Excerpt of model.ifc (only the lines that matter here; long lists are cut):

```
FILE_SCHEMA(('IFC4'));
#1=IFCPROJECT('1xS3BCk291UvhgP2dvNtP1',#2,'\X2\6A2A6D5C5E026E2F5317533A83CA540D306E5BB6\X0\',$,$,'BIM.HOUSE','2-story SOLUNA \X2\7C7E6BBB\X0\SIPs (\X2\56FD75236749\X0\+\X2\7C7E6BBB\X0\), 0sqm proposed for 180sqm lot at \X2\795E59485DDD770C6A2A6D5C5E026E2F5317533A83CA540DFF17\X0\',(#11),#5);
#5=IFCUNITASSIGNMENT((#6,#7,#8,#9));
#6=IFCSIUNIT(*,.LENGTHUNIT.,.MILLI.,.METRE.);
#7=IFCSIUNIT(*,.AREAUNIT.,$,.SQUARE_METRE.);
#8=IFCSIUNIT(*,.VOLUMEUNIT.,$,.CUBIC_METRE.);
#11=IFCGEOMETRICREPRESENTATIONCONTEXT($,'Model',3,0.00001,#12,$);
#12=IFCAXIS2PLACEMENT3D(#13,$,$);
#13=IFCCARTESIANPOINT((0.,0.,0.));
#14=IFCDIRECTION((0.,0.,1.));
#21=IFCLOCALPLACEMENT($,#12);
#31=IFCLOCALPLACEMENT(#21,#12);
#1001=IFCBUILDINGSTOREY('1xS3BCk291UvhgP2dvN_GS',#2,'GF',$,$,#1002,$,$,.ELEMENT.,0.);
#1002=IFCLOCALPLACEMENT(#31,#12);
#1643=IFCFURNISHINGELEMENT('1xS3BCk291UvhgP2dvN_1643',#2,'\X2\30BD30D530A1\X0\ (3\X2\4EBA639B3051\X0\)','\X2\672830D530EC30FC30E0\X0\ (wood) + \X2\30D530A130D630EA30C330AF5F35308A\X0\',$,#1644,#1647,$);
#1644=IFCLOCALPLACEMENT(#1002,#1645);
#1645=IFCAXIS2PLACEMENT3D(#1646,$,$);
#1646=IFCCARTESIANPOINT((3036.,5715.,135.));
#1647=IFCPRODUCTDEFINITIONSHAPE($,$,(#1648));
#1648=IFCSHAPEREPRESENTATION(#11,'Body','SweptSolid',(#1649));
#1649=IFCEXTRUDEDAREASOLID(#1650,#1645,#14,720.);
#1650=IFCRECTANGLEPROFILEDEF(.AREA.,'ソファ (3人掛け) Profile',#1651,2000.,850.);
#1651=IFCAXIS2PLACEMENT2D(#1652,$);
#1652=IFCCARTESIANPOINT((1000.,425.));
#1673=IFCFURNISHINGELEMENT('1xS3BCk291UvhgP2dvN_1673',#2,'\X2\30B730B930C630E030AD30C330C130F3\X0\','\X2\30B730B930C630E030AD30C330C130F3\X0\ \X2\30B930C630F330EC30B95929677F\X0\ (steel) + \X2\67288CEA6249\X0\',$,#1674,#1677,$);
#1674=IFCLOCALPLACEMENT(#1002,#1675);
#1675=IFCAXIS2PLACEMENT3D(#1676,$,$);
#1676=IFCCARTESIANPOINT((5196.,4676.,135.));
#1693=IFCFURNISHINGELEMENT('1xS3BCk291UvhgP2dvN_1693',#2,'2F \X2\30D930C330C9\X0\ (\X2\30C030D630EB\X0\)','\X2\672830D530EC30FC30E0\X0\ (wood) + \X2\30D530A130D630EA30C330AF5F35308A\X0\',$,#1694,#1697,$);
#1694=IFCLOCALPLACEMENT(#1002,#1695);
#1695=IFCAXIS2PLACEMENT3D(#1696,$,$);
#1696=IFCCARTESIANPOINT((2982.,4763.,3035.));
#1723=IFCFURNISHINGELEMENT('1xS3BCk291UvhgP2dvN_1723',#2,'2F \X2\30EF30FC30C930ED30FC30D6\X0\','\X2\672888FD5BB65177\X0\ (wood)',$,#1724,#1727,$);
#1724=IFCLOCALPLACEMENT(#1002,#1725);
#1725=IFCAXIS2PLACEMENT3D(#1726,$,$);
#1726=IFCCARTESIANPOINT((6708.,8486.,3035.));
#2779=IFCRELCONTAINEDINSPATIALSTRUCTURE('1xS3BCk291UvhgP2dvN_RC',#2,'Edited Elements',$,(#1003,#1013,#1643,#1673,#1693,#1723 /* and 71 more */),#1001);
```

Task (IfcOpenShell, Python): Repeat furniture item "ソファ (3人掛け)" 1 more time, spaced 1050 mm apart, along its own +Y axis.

```python
import ifcopenshell
import ifcopenshell.api.geometry
import ifcopenshell.api.root
import ifcopenshell.util.element
import ifcopenshell.util.placement
import ifcopenshell.util.unit

model = ifcopenshell.open("model.ifc")
unit_scale = ifcopenshell.util.unit.calculate_unit_scale(model)


def reuse_history(source, copy):
    """copy_class also copies each property set's owner history, people and application; keep the originals."""
    for rel in copy.IsDefinedBy:
        if rel.is_a("IfcRelDefinesByProperties") and (history := rel.RelatingPropertyDefinition.OwnerHistory):
            rel.RelatingPropertyDefinition.OwnerHistory = source.OwnerHistory
            ifcopenshell.util.element.remove_deep2(model, history)


source = model.by_guid("1xS3BCk291UvhgP2dvN_1643")
base = ifcopenshell.util.placement.get_local_placement(source.ObjectPlacement)
step = base[:3, 1] * 1.05 / unit_scale

for i in range(1, 2):
    copy = ifcopenshell.api.root.copy_class(model, product=source)
    copy.Representation = ifcopenshell.util.element.copy_deep(
        model, source.Representation, exclude=["IfcGeometricRepresentationContext", "IfcRepresentationMap"]
    )
    reuse_history(source, copy)
    matrix = base.copy()
    matrix[:3, 3] += i * step
    print("added at", matrix[:3, 3].round(3) + 0.0)
    ifcopenshell.api.geometry.edit_object_placement(model, product=copy, matrix=matrix, is_si=False)

model.write("model_updated.ifc")
```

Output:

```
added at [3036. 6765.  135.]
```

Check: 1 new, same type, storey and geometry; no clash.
